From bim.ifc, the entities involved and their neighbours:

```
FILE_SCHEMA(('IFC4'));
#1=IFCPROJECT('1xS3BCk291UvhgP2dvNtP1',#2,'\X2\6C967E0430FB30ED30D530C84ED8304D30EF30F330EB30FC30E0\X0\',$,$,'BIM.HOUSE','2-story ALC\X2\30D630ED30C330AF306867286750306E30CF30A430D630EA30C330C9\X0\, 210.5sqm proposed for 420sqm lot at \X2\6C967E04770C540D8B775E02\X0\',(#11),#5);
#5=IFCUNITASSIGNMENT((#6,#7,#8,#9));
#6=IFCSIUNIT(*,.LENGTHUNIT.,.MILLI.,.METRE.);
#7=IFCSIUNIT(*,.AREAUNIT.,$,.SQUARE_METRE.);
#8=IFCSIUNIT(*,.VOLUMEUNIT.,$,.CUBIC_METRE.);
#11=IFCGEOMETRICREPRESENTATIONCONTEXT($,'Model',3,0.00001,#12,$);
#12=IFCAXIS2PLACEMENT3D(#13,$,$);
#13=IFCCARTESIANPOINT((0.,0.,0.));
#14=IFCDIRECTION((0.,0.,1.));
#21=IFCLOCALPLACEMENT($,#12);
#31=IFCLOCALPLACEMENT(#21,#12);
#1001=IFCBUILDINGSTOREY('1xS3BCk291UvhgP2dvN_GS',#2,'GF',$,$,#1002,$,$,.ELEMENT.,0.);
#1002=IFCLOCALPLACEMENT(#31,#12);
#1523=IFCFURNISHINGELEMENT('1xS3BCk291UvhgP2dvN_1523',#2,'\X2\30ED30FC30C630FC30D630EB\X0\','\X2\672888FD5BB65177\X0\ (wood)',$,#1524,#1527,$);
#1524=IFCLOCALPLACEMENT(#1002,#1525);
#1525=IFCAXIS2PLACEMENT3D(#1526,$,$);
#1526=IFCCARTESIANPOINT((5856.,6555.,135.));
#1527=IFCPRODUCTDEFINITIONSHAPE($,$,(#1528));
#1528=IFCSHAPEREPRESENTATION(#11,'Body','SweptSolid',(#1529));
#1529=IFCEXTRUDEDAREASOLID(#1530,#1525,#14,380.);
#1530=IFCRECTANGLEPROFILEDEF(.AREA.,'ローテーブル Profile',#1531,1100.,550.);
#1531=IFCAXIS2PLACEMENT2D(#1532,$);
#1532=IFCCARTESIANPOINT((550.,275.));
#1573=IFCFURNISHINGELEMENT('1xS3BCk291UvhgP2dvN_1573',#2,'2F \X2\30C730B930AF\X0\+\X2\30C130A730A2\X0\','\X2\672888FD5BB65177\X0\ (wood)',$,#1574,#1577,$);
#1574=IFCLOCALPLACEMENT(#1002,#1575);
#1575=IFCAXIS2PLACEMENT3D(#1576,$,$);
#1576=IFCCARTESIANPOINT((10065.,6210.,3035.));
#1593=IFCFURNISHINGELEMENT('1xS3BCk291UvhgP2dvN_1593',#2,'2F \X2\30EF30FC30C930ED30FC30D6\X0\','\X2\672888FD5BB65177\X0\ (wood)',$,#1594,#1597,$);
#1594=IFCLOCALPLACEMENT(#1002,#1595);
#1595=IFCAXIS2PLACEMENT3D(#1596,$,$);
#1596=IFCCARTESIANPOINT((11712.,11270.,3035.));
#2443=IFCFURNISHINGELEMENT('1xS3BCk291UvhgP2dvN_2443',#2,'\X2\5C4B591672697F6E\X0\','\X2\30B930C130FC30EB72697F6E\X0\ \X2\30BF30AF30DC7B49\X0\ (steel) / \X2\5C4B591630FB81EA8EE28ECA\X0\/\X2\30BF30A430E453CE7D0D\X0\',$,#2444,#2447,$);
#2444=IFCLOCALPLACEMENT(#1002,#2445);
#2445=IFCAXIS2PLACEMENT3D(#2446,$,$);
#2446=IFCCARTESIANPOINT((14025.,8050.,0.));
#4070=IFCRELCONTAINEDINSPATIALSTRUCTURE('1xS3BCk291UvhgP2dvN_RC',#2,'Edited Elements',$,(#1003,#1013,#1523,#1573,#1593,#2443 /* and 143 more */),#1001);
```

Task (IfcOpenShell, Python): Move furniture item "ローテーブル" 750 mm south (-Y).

```python
import ifcopenshell
import ifcopenshell.api.geometry
import ifcopenshell.util.placement

model = ifcopenshell.open("bim.ifc")

item = model.by_guid("1xS3BCk291UvhgP2dvN_1523")
matrix = ifcopenshell.util.placement.get_local_placement(item.ObjectPlacement)
matrix[1, 3] -= 750.0
ifcopenshell.api.geometry.edit_object_placement(model, product=item, matrix=matrix, is_si=False)

print(ifcopenshell.util.placement.get_local_placement(item.ObjectPlacement).round(3) + 0.0)

model.write("bim-out.ifc")
```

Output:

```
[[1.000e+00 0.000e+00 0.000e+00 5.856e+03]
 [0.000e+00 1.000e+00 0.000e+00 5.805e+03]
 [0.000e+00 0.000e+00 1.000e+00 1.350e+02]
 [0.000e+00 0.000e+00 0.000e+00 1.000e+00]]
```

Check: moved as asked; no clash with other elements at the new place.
